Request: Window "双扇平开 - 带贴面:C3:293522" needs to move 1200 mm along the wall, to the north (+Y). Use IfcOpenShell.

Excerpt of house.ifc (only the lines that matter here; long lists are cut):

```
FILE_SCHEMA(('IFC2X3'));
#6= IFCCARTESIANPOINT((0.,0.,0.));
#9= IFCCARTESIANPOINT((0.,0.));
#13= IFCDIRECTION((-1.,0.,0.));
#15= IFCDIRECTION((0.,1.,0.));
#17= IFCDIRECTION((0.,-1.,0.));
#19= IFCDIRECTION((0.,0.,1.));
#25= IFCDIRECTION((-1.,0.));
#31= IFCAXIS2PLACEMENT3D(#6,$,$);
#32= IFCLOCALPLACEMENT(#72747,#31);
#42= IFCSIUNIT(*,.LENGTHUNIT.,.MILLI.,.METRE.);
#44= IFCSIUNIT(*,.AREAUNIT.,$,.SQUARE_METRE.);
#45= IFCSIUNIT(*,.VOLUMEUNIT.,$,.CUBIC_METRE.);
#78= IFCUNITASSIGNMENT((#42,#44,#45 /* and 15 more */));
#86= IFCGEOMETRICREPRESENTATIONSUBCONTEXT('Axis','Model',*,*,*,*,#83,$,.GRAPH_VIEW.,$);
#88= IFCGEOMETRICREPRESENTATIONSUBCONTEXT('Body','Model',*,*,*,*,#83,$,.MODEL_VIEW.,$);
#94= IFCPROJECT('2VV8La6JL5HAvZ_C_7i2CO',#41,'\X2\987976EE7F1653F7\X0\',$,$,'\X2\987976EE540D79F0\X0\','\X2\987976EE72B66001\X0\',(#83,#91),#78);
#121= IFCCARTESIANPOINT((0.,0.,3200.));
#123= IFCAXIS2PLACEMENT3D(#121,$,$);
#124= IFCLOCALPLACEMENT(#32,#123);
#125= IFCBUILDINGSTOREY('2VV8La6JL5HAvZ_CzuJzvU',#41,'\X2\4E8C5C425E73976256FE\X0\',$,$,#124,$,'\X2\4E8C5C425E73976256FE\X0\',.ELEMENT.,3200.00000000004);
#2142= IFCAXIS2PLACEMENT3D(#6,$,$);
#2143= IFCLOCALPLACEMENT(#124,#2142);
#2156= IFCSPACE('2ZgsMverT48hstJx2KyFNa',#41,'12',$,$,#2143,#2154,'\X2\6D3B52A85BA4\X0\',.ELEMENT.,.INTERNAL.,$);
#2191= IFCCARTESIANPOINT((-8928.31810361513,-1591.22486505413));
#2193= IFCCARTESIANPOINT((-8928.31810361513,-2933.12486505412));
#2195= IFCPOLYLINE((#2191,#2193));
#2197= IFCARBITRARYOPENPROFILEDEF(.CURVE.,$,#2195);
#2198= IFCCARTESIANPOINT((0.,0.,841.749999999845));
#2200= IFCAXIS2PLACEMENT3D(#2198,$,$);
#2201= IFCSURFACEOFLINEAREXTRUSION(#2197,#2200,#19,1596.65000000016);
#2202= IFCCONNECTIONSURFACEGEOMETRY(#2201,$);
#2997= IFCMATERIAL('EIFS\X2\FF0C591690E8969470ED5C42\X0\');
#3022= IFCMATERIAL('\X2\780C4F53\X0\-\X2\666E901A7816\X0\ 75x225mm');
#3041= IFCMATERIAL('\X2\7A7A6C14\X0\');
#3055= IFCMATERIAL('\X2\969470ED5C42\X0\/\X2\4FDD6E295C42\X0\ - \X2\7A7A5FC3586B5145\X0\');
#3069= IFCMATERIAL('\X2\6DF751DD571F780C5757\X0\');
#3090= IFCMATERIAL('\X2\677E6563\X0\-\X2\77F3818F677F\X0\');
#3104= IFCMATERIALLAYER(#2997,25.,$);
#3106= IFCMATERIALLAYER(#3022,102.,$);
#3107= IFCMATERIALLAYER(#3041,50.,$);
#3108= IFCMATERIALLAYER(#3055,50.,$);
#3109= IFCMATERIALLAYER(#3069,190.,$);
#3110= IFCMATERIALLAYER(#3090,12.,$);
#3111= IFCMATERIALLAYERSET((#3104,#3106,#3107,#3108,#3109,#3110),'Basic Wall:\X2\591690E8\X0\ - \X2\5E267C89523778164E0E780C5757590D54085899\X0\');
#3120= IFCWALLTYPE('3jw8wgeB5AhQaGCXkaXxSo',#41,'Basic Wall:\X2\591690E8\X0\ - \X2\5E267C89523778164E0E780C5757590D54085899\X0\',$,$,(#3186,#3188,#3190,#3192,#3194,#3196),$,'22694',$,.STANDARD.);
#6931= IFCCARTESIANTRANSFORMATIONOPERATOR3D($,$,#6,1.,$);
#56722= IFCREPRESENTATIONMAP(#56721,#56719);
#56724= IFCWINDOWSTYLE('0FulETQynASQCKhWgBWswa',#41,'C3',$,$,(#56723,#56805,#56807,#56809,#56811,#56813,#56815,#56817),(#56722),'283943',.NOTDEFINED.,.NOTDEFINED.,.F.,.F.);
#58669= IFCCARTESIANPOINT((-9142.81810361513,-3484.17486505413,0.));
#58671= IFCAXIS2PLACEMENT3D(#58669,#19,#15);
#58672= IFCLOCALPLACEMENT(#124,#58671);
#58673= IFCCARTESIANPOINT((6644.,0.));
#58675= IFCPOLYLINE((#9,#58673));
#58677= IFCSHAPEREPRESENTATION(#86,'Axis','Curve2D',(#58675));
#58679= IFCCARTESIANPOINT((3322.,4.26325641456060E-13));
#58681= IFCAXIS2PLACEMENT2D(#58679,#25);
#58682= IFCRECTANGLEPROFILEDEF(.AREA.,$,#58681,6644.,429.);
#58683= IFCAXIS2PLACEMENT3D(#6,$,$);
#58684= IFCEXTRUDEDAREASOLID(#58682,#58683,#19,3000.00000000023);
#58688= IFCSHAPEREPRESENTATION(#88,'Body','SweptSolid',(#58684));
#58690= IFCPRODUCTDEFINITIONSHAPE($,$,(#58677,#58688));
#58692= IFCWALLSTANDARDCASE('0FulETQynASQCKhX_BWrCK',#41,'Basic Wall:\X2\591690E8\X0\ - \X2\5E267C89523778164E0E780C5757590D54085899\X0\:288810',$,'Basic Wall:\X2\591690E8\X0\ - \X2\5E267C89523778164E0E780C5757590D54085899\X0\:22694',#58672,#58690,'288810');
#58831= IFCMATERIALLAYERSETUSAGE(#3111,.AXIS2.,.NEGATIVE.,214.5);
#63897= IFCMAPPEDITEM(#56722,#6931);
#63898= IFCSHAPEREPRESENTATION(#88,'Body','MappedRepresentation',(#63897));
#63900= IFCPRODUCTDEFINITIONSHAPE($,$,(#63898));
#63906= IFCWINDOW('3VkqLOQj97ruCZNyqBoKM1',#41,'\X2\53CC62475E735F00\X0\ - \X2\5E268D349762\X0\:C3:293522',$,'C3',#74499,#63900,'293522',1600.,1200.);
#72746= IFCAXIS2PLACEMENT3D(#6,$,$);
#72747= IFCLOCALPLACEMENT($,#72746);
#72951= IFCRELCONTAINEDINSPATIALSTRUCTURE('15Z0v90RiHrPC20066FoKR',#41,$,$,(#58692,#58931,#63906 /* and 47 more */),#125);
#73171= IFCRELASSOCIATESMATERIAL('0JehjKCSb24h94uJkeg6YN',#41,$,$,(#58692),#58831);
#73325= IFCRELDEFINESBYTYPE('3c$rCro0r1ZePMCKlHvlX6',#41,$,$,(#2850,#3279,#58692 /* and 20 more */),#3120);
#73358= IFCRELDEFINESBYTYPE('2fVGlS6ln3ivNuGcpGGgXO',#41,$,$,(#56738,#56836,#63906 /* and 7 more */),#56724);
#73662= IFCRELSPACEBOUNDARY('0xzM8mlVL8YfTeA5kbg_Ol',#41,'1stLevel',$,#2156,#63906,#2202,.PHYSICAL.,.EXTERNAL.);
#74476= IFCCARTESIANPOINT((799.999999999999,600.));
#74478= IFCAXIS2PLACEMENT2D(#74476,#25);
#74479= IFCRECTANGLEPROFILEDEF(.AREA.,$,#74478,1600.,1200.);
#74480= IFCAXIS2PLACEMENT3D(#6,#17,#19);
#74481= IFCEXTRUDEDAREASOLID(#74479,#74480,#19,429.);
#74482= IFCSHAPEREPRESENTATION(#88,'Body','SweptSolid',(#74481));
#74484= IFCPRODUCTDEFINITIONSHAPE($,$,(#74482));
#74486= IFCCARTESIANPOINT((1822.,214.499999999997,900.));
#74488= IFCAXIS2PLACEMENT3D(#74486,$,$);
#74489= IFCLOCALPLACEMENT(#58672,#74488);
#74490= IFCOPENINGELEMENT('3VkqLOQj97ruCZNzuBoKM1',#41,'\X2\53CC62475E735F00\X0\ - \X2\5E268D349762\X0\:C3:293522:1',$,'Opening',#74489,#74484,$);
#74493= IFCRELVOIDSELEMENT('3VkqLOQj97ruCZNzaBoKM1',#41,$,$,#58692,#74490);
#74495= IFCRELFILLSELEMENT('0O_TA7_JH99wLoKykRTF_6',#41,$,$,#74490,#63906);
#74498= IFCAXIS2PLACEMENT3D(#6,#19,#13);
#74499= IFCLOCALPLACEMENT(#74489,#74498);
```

```python
import numpy as np
import ifcopenshell
import ifcopenshell.api.geometry
import ifcopenshell.util.placement
import ifcopenshell.util.unit

model = ifcopenshell.open("house.ifc")
unit_scale = ifcopenshell.util.unit.calculate_unit_scale(model)

window = model.by_id(63906)
opening = window.FillsVoids[0].RelatingOpeningElement
wall = opening.VoidsElements[0].RelatingBuildingElement

wall_matrix = ifcopenshell.util.placement.get_local_placement(wall.ObjectPlacement)
shift = wall_matrix[:3, 0] * 1.2 / unit_scale
before = ifcopenshell.util.placement.get_local_placement(window.ObjectPlacement)[:3, 3].copy()

# The window is placed relative to its opening, so it follows when the opening moves.
matrix = ifcopenshell.util.placement.get_local_placement(opening.ObjectPlacement)
matrix[:3, 3] += shift
ifcopenshell.api.geometry.edit_object_placement(
    model, product=opening, matrix=matrix, is_si=False, should_transform_children=True
)

# Space boundary surfaces are stored in each space's coordinates; move them too.
for rel in window.ProvidesBoundaries:
    if not rel.ConnectionGeometry:
        continue
    surface = rel.ConnectionGeometry.SurfaceOnRelatingElement
    space_matrix = ifcopenshell.util.placement.get_local_placement(rel.RelatingSpace.ObjectPlacement)
    point = np.array(surface.Position.Location.Coordinates) + space_matrix[:3, :3].T @ shift
    surface.Position = model.createIfcAxis2Placement3D(
        model.createIfcCartesianPoint(point.tolist()), surface.Position.Axis, surface.Position.RefDirection
    )

after = ifcopenshell.util.placement.get_local_placement(window.ObjectPlacement)[:3, 3]
print("window moved by", (after - before).round(3) + 0.0)

model.write("house_updated.ifc")
```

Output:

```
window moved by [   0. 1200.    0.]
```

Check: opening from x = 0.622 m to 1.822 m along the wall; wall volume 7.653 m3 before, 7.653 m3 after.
